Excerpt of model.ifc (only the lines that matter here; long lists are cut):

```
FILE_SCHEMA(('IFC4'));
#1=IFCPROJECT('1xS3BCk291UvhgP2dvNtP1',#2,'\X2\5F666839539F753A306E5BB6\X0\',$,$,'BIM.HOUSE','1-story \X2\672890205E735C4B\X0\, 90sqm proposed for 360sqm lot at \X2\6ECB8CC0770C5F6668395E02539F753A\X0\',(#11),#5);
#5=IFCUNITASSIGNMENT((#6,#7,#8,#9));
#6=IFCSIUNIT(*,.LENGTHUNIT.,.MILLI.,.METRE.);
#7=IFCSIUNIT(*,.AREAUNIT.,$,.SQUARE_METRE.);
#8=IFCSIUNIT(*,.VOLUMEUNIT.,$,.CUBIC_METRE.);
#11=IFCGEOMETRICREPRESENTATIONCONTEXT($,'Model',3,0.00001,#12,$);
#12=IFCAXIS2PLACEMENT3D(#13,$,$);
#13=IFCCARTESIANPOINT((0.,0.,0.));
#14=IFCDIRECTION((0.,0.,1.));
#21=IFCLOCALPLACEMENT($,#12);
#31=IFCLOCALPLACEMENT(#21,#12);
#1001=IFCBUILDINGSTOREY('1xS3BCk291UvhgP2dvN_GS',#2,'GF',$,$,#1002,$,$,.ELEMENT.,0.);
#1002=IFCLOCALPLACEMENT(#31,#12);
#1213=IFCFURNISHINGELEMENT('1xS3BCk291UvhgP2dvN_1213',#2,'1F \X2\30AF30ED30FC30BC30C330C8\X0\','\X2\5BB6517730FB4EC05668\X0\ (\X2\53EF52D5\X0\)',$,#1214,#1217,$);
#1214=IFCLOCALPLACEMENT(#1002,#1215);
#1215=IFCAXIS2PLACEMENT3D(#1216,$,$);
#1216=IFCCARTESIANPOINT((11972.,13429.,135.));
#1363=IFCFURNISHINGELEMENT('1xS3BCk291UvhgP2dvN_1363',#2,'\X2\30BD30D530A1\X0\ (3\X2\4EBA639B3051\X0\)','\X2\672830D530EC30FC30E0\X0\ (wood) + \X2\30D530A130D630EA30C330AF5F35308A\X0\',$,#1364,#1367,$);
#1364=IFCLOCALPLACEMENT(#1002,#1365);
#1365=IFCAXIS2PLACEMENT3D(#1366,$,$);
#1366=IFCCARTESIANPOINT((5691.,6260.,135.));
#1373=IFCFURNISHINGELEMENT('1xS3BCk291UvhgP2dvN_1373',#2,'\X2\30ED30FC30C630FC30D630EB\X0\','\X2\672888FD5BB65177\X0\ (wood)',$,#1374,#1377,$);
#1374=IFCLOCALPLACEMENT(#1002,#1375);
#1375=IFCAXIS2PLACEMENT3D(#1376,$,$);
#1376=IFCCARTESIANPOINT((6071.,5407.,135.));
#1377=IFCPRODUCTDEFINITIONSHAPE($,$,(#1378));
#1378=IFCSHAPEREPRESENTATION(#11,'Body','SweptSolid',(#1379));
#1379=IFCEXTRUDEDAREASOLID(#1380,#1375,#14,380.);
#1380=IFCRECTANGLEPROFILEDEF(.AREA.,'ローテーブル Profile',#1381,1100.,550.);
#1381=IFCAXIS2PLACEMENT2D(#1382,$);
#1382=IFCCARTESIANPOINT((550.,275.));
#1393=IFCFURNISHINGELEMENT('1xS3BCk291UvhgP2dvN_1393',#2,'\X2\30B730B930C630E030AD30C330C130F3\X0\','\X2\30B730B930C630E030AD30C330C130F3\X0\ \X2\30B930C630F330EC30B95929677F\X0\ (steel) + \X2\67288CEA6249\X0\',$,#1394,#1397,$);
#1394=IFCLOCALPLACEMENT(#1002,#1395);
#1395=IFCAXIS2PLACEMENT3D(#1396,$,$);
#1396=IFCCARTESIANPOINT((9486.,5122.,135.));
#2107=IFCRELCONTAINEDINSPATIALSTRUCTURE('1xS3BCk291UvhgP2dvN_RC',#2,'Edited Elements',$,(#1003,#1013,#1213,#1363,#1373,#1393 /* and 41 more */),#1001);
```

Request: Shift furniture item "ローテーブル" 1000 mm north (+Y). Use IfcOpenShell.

```python
import ifcopenshell
import ifcopenshell.api.geometry
import ifcopenshell.util.placement
import ifcopenshell.util.unit

model = ifcopenshell.open("model.ifc")
unit_scale = ifcopenshell.util.unit.calculate_unit_scale(model)

item = model.by_guid("1xS3BCk291UvhgP2dvN_1373")
matrix = ifcopenshell.util.placement.get_local_placement(item.ObjectPlacement)
matrix[1, 3] += 1 / unit_scale
ifcopenshell.api.geometry.edit_object_placement(model, product=item, matrix=matrix, is_si=False)

print(ifcopenshell.util.placement.get_local_placement(item.ObjectPlacement).round(3) + 0.0)

model.write("model_updated.ifc")
```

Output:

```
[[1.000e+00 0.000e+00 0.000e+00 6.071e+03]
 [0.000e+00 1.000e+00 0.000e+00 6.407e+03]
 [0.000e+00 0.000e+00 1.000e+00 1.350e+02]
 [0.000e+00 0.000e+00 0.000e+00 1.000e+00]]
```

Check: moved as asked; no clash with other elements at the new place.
